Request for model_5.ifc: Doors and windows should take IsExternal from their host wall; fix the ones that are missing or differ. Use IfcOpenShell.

First a look at what the model holds.

```python
import ifcopenshell
import ifcopenshell.util.element

model = ifcopenshell.open("model_5.ifc")
print(model.schema)
seen = {}
for e in model.by_type("IfcDoor") + model.by_type("IfcWindow"):
    if not e.FillsVoids:
        continue
    host = e.FillsVoids[0].RelatingOpeningElement.VoidsElements[0].RelatingBuildingElement
    own = ifcopenshell.util.element.get_pset(e, f"Pset_{e.is_a()[3:].removesuffix('StandardCase')}Common", "IsExternal")
    wall = ifcopenshell.util.element.get_pset(host, "Pset_WallCommon", "IsExternal")
    seen[e.is_a(), own, wall] = seen.get((e.is_a(), own, wall), 0) + 1
for (cls, own, wall), count in sorted(seen.items(), key=str):
    print(count, cls, "IsExternal:", own, "| host wall:", wall)
```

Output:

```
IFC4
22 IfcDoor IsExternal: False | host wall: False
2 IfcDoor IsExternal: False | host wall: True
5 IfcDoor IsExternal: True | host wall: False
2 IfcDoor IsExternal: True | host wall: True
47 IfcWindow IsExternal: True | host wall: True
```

```python
import ifcopenshell
import ifcopenshell.api.pset
import ifcopenshell.util.element

model = ifcopenshell.open("model_5.ifc")

count = 0
for ifc_class, pset_name in (("IfcDoor", "Pset_DoorCommon"), ("IfcWindow", "Pset_WindowCommon")):
    for e in model.by_type(ifc_class):
        if not e.FillsVoids:
            continue
        host = e.FillsVoids[0].RelatingOpeningElement.VoidsElements[0].RelatingBuildingElement
        external = ifcopenshell.util.element.get_pset(host, "Pset_WallCommon", "IsExternal")
        if external is None or ifcopenshell.util.element.get_pset(e, pset_name, "IsExternal") == external:
            continue
        pset = ifcopenshell.api.pset.add_pset(model, product=e, name=pset_name)
        ifcopenshell.api.pset.edit_pset(model, pset=pset, properties={"IsExternal": external})
        count += 1

print(count, "updated")

model.write("model_5_rev.ifc")
```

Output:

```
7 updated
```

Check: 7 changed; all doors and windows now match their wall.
